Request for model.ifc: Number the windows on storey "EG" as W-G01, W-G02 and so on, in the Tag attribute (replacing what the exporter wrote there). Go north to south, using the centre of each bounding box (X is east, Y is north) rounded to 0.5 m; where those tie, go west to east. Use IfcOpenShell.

First a look at what the model holds.

```python
import ifcopenshell
import ifcopenshell.util.element
import ifcopenshell.util.placement

model = ifcopenshell.open("model.ifc")
print(model.schema)
storey = next(s for s in model.by_type("IfcBuildingStorey") if s.Name == "EG")
windows = [e for e in ifcopenshell.util.element.get_decomposition(storey) if e.is_a("IfcWindow")]
for e in sorted(windows, key=lambda e: e.id()):
    origin = ifcopenshell.util.placement.get_local_placement(e.ObjectPlacement)[:3, 3]
    print(e.id(), e.Tag, e.Name, origin.round(2) + 0.0, sep=" | ")
```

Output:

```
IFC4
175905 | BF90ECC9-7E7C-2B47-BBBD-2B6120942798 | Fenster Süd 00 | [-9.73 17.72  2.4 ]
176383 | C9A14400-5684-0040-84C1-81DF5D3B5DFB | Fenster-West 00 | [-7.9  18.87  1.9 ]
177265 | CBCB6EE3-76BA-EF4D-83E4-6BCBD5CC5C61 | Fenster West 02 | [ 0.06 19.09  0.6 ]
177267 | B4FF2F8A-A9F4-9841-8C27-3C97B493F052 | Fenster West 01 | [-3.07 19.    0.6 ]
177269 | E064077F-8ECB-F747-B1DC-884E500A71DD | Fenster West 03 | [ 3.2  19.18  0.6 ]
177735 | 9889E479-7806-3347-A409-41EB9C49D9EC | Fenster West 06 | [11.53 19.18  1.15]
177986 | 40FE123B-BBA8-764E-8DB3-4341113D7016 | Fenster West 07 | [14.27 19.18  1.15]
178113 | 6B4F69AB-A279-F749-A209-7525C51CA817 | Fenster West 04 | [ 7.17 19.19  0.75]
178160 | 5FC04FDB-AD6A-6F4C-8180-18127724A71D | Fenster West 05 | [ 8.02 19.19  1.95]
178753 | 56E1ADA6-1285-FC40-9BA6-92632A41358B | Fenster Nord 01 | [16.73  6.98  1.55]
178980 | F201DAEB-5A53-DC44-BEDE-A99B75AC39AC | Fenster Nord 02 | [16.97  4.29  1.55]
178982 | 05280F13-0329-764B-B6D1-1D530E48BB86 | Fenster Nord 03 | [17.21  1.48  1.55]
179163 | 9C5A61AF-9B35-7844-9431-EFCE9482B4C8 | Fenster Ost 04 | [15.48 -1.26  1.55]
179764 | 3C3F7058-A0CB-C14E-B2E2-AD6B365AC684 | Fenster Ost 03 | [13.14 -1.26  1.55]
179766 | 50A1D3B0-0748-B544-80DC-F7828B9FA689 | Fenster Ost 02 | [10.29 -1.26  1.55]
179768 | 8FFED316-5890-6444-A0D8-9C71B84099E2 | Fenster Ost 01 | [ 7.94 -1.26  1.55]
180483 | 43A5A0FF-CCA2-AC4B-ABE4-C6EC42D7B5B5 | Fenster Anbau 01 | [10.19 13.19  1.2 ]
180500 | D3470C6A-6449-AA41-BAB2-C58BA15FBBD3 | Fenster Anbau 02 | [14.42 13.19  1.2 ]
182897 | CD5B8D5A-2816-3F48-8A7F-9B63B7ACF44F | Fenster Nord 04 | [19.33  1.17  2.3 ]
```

```python
import ifcopenshell
import ifcopenshell.geom
import ifcopenshell.util.element
import ifcopenshell.util.shape

model = ifcopenshell.open("model.ifc")
settings = ifcopenshell.geom.settings()
settings.set("use-world-coords", True)


def centre(element):
    shape = ifcopenshell.geom.create_shape(settings, element)
    return ifcopenshell.util.shape.get_bbox_centroid(shape.geometry)


storey = next(s for s in model.by_type("IfcBuildingStorey") if s.Name == "EG")
windows = [e for e in ifcopenshell.util.element.get_decomposition(storey) if e.is_a("IfcWindow")]

# Insertion points can sit at a corner or the storey origin, so sort by the geometry (in metres).
centres = {e: centre(e) for e in windows}
windows.sort(key=lambda e: (-round(centres[e][1] / 0.5), centres[e][0]))

for i, e in enumerate(windows, start=1):
    number = f"W-G{i:02d}"
    e.Tag = number
    print(e.id(), number)

model.write("model_updated.ifc")
```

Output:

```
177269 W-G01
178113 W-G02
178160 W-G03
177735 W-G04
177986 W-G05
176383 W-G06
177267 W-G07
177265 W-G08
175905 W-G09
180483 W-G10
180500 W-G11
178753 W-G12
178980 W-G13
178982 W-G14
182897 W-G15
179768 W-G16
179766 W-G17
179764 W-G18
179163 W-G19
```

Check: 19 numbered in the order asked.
